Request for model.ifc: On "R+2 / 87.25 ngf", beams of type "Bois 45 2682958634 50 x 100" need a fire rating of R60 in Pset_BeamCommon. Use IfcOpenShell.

First a look at what the model holds.

```python
import ifcopenshell
import ifcopenshell.util.element

model = ifcopenshell.open("model.ifc")
print(model.schema)
storey = next(s for s in model.by_type("IfcBuildingStorey") if s.Name == "R+2 / 87.25 ngf")
beams = [e for e in ifcopenshell.util.element.get_decomposition(storey) if e.is_a("IfcBeam")]
seen = {}
for e in beams:
    element_type = ifcopenshell.util.element.get_type(e)
    key = (element_type.Name if element_type != e and element_type else None, ifcopenshell.util.element.get_pset(e, "Pset_BeamCommon", "FireRating"))
    seen[key] = seen.get(key, 0) + 1
for (name, value), count in sorted(seen.items(), key=str):
    print(count, "x", name, "|", value)
```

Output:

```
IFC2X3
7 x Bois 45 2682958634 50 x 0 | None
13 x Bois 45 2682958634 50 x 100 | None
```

```python
import ifcopenshell
import ifcopenshell.api.pset
import ifcopenshell.util.element

model = ifcopenshell.open("model.ifc")

storey = next(s for s in model.by_type("IfcBuildingStorey") if s.Name == "R+2 / 87.25 ngf")
beams = [e for e in ifcopenshell.util.element.get_decomposition(storey) if e.is_a("IfcBeam")]

count = 0
for e in beams:
    element_type = ifcopenshell.util.element.get_type(e)
    if element_type in (None, e) or element_type.Name != "Bois 45 2682958634 50 x 100":
        continue
    # add_pset returns the element's existing set when there is one.
    pset = ifcopenshell.api.pset.add_pset(model, product=e, name="Pset_BeamCommon")
    ifcopenshell.api.pset.edit_pset(model, pset=pset, properties={"FireRating": "R60"})
    count += 1

print(count, "beams updated")

model.write("model_v2.ifc")
```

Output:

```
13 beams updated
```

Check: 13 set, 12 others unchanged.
